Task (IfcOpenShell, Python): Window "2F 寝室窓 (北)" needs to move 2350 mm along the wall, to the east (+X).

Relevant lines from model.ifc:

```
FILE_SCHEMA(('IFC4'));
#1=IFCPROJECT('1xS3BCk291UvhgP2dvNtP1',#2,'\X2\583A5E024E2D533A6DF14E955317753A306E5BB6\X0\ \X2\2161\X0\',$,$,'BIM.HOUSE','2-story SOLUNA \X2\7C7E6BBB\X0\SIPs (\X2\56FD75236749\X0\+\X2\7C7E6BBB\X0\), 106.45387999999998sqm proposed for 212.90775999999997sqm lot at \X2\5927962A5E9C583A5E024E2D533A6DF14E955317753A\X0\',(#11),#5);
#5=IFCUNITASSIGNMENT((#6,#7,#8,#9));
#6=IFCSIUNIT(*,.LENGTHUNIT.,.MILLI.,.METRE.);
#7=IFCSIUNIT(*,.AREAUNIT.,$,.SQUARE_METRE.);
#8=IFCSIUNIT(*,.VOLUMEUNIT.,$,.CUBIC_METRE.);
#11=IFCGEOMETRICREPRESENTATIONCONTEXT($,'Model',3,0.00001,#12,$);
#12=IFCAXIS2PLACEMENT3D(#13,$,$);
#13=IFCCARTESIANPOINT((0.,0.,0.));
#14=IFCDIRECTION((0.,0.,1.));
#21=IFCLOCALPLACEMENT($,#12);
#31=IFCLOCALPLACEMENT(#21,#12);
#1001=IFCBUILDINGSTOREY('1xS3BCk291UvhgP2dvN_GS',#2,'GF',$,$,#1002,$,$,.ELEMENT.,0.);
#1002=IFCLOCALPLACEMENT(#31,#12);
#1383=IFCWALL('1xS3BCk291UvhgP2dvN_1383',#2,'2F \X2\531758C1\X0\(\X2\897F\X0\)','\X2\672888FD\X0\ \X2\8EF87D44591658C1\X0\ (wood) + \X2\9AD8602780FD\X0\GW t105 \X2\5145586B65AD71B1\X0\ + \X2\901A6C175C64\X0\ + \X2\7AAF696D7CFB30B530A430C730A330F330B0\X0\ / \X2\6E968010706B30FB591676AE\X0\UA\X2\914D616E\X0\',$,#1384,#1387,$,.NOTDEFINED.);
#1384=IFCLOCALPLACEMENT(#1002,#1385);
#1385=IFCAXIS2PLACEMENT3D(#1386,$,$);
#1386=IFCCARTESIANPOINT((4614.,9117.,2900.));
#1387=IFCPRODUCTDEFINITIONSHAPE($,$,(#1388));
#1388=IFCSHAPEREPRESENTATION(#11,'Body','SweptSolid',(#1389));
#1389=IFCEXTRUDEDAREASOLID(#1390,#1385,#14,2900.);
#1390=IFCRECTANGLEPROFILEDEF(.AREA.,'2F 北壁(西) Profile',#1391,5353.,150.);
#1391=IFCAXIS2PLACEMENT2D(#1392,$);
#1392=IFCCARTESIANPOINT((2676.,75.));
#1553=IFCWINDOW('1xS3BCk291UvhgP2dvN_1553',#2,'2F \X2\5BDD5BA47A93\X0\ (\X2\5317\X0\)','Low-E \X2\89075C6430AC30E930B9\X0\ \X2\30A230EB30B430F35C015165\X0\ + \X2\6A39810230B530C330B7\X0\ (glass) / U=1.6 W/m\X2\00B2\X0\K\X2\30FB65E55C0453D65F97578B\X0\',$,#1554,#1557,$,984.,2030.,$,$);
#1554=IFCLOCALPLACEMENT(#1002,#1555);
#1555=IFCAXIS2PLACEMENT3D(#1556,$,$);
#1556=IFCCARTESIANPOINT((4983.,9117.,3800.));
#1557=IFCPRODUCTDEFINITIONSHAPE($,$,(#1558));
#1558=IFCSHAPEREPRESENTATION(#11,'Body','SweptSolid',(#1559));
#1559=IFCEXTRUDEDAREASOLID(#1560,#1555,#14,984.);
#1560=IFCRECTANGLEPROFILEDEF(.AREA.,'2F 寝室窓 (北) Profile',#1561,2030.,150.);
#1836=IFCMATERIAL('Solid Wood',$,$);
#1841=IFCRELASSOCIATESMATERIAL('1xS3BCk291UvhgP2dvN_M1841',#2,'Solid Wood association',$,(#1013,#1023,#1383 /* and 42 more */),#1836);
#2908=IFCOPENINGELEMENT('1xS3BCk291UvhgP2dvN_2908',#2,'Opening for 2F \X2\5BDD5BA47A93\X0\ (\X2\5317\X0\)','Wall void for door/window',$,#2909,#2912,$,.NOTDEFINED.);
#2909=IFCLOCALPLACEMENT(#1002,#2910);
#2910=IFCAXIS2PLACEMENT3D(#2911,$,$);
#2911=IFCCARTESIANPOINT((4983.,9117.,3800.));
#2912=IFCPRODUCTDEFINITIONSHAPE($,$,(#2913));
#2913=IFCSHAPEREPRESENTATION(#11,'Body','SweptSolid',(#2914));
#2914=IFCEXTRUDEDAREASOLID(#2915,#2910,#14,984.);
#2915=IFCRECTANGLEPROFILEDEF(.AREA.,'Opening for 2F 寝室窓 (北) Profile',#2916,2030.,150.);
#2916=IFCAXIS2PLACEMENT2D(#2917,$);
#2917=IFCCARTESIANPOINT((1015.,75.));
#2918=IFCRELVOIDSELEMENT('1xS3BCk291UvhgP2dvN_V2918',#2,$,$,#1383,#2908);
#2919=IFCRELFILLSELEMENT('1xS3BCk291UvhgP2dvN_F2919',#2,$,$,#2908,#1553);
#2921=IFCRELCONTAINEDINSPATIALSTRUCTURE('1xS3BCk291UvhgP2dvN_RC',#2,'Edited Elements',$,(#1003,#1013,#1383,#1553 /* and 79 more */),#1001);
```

```python
import ifcopenshell
import ifcopenshell.api.geometry
import ifcopenshell.util.placement

model = ifcopenshell.open("model.ifc")

window = model.by_id(1553)
opening = window.FillsVoids[0].RelatingOpeningElement
wall = opening.VoidsElements[0].RelatingBuildingElement

wall_matrix = ifcopenshell.util.placement.get_local_placement(wall.ObjectPlacement)
shift = wall_matrix[:3, 0] * 2350.0
before = ifcopenshell.util.placement.get_local_placement(window.ObjectPlacement)[:3, 3].copy()

# The window is not placed relative to its opening, so move both.
for product in (opening, window):
    matrix = ifcopenshell.util.placement.get_local_placement(product.ObjectPlacement)
    matrix[:3, 3] += shift
    ifcopenshell.api.geometry.edit_object_placement(model, product=product, matrix=matrix, is_si=False)

after = ifcopenshell.util.placement.get_local_placement(window.ObjectPlacement)[:3, 3]
print("window moved by", (after - before).round(3) + 0.0)

model.write("model_updated.ifc")
```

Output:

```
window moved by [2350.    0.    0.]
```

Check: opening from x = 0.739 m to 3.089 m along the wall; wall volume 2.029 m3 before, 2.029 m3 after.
